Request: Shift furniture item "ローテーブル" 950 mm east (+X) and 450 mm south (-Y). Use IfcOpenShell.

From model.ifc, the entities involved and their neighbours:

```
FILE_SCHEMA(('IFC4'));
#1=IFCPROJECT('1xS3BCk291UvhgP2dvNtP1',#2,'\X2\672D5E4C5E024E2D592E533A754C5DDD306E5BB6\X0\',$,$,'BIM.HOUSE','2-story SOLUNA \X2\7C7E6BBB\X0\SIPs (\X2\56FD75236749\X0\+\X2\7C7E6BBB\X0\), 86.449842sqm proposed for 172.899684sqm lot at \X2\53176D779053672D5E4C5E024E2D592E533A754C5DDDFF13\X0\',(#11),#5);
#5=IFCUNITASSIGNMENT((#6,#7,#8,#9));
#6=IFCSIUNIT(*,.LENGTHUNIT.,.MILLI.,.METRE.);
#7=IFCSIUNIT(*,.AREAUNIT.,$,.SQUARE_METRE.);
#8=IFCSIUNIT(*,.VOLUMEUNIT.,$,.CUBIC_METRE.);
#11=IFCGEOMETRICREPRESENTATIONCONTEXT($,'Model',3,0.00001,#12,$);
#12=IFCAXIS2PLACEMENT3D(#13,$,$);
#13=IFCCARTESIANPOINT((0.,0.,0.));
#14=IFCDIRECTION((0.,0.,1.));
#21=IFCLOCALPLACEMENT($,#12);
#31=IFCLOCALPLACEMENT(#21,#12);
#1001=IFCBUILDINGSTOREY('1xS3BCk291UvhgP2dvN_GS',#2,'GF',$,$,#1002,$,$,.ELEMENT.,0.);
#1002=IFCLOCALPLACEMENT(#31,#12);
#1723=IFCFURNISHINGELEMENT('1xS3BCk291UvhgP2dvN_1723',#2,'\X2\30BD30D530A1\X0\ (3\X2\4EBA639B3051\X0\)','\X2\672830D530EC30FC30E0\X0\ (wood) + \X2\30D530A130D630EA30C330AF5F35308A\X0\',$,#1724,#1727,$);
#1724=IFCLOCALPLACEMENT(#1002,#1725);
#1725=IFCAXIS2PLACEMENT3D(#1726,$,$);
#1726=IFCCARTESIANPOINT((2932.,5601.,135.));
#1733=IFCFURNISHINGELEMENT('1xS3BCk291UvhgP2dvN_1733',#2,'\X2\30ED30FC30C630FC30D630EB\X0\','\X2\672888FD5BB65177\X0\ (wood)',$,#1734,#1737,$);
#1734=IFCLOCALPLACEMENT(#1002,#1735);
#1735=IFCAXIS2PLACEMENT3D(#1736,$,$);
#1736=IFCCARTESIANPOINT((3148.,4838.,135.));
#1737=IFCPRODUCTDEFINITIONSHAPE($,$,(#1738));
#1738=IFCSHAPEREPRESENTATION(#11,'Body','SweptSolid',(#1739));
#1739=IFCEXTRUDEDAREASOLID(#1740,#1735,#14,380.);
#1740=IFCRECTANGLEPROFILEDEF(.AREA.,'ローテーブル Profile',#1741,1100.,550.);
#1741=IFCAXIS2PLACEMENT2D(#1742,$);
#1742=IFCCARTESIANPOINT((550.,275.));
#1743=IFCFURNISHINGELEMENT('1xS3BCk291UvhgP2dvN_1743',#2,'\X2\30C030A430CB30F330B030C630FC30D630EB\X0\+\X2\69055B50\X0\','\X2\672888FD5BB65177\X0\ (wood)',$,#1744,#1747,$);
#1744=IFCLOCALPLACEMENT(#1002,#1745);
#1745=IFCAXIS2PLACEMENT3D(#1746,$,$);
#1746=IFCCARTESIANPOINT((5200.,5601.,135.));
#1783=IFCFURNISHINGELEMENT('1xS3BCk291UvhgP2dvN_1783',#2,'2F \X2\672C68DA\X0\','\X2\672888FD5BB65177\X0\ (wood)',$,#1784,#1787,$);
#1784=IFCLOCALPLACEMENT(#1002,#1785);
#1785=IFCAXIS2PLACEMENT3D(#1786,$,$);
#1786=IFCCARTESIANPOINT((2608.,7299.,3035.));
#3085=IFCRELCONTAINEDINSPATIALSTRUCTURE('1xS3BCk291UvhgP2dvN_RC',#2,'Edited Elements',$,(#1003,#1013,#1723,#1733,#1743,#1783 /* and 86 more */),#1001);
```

```python
import ifcopenshell
import ifcopenshell.api.geometry
import ifcopenshell.util.placement

model = ifcopenshell.open("model.ifc")

item = model.by_id(1733)
matrix = ifcopenshell.util.placement.get_local_placement(item.ObjectPlacement)
matrix[0, 3] += 950.0
matrix[1, 3] -= 450.0
ifcopenshell.api.geometry.edit_object_placement(model, product=item, matrix=matrix, is_si=False)

print(ifcopenshell.util.placement.get_local_placement(item.ObjectPlacement).round(3) + 0.0)

model.write("model-out.ifc")
```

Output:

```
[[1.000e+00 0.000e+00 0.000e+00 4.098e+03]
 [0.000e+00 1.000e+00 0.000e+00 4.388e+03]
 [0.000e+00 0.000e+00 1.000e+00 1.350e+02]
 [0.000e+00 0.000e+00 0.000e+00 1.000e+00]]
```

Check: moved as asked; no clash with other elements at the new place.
